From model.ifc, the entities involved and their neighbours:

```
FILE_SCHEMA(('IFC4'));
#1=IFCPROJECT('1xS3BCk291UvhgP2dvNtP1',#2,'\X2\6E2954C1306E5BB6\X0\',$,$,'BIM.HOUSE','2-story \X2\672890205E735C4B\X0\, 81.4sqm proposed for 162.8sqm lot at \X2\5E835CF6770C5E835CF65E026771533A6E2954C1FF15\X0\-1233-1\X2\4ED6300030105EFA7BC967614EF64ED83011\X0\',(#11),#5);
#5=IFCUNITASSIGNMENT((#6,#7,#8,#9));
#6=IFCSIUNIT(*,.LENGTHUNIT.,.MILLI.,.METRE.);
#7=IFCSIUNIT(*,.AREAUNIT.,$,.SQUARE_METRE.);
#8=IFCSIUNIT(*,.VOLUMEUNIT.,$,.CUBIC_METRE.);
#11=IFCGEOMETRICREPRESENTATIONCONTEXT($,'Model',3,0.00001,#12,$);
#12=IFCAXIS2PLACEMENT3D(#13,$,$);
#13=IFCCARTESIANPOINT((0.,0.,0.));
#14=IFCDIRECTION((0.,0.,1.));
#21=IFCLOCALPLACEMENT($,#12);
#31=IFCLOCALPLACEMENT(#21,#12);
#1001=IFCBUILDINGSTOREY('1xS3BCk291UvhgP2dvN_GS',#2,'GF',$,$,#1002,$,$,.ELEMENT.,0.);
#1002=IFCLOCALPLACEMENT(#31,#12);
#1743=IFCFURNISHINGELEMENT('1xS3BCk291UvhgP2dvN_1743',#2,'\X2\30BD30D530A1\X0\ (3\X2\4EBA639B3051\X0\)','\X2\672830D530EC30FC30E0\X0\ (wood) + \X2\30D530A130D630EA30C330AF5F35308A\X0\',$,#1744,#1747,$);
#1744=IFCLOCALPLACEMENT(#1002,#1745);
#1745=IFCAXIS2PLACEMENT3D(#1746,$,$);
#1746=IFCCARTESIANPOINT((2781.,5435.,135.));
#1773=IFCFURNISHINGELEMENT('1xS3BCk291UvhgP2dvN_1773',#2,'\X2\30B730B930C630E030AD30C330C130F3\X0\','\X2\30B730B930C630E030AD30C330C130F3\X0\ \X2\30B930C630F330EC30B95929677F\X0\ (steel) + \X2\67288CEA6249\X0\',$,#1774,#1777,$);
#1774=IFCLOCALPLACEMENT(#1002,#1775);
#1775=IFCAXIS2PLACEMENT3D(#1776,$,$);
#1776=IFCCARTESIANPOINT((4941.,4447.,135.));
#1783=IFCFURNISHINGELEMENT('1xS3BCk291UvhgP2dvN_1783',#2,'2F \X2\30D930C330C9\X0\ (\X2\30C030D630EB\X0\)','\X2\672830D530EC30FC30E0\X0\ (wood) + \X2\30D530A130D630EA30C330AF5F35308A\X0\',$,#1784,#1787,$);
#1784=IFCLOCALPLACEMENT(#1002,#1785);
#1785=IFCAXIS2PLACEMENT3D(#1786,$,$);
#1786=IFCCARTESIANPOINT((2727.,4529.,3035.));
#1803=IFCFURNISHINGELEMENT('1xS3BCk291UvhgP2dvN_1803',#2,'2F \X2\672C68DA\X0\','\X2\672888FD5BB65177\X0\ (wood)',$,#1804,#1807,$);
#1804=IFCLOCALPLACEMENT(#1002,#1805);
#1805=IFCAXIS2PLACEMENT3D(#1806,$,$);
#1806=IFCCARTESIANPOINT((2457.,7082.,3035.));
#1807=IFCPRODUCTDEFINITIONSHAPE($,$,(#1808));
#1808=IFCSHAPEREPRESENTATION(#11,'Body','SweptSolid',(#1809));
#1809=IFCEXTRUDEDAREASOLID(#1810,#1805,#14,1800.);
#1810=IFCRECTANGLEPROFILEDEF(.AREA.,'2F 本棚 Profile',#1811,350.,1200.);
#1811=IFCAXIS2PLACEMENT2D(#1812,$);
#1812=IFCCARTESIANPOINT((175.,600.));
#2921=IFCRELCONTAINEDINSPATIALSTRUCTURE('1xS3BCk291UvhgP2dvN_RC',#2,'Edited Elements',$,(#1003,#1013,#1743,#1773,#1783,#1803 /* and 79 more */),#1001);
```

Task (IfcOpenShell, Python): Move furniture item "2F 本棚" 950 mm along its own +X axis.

```python
import ifcopenshell
import ifcopenshell.api.geometry
import ifcopenshell.util.placement
import ifcopenshell.util.unit

model = ifcopenshell.open("model.ifc")
unit_scale = ifcopenshell.util.unit.calculate_unit_scale(model)

item = model.by_guid("1xS3BCk291UvhgP2dvN_1803")
matrix = ifcopenshell.util.placement.get_local_placement(item.ObjectPlacement)
matrix[:3, 3] += matrix[:3, 0] * 0.95 / unit_scale
ifcopenshell.api.geometry.edit_object_placement(model, product=item, matrix=matrix, is_si=False)

print(ifcopenshell.util.placement.get_local_placement(item.ObjectPlacement).round(3) + 0.0)

model.write("model_updated.ifc")
```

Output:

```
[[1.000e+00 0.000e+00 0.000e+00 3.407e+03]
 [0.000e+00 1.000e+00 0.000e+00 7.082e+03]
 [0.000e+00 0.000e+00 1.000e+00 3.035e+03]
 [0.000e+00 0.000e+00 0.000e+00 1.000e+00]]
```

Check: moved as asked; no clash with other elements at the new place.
